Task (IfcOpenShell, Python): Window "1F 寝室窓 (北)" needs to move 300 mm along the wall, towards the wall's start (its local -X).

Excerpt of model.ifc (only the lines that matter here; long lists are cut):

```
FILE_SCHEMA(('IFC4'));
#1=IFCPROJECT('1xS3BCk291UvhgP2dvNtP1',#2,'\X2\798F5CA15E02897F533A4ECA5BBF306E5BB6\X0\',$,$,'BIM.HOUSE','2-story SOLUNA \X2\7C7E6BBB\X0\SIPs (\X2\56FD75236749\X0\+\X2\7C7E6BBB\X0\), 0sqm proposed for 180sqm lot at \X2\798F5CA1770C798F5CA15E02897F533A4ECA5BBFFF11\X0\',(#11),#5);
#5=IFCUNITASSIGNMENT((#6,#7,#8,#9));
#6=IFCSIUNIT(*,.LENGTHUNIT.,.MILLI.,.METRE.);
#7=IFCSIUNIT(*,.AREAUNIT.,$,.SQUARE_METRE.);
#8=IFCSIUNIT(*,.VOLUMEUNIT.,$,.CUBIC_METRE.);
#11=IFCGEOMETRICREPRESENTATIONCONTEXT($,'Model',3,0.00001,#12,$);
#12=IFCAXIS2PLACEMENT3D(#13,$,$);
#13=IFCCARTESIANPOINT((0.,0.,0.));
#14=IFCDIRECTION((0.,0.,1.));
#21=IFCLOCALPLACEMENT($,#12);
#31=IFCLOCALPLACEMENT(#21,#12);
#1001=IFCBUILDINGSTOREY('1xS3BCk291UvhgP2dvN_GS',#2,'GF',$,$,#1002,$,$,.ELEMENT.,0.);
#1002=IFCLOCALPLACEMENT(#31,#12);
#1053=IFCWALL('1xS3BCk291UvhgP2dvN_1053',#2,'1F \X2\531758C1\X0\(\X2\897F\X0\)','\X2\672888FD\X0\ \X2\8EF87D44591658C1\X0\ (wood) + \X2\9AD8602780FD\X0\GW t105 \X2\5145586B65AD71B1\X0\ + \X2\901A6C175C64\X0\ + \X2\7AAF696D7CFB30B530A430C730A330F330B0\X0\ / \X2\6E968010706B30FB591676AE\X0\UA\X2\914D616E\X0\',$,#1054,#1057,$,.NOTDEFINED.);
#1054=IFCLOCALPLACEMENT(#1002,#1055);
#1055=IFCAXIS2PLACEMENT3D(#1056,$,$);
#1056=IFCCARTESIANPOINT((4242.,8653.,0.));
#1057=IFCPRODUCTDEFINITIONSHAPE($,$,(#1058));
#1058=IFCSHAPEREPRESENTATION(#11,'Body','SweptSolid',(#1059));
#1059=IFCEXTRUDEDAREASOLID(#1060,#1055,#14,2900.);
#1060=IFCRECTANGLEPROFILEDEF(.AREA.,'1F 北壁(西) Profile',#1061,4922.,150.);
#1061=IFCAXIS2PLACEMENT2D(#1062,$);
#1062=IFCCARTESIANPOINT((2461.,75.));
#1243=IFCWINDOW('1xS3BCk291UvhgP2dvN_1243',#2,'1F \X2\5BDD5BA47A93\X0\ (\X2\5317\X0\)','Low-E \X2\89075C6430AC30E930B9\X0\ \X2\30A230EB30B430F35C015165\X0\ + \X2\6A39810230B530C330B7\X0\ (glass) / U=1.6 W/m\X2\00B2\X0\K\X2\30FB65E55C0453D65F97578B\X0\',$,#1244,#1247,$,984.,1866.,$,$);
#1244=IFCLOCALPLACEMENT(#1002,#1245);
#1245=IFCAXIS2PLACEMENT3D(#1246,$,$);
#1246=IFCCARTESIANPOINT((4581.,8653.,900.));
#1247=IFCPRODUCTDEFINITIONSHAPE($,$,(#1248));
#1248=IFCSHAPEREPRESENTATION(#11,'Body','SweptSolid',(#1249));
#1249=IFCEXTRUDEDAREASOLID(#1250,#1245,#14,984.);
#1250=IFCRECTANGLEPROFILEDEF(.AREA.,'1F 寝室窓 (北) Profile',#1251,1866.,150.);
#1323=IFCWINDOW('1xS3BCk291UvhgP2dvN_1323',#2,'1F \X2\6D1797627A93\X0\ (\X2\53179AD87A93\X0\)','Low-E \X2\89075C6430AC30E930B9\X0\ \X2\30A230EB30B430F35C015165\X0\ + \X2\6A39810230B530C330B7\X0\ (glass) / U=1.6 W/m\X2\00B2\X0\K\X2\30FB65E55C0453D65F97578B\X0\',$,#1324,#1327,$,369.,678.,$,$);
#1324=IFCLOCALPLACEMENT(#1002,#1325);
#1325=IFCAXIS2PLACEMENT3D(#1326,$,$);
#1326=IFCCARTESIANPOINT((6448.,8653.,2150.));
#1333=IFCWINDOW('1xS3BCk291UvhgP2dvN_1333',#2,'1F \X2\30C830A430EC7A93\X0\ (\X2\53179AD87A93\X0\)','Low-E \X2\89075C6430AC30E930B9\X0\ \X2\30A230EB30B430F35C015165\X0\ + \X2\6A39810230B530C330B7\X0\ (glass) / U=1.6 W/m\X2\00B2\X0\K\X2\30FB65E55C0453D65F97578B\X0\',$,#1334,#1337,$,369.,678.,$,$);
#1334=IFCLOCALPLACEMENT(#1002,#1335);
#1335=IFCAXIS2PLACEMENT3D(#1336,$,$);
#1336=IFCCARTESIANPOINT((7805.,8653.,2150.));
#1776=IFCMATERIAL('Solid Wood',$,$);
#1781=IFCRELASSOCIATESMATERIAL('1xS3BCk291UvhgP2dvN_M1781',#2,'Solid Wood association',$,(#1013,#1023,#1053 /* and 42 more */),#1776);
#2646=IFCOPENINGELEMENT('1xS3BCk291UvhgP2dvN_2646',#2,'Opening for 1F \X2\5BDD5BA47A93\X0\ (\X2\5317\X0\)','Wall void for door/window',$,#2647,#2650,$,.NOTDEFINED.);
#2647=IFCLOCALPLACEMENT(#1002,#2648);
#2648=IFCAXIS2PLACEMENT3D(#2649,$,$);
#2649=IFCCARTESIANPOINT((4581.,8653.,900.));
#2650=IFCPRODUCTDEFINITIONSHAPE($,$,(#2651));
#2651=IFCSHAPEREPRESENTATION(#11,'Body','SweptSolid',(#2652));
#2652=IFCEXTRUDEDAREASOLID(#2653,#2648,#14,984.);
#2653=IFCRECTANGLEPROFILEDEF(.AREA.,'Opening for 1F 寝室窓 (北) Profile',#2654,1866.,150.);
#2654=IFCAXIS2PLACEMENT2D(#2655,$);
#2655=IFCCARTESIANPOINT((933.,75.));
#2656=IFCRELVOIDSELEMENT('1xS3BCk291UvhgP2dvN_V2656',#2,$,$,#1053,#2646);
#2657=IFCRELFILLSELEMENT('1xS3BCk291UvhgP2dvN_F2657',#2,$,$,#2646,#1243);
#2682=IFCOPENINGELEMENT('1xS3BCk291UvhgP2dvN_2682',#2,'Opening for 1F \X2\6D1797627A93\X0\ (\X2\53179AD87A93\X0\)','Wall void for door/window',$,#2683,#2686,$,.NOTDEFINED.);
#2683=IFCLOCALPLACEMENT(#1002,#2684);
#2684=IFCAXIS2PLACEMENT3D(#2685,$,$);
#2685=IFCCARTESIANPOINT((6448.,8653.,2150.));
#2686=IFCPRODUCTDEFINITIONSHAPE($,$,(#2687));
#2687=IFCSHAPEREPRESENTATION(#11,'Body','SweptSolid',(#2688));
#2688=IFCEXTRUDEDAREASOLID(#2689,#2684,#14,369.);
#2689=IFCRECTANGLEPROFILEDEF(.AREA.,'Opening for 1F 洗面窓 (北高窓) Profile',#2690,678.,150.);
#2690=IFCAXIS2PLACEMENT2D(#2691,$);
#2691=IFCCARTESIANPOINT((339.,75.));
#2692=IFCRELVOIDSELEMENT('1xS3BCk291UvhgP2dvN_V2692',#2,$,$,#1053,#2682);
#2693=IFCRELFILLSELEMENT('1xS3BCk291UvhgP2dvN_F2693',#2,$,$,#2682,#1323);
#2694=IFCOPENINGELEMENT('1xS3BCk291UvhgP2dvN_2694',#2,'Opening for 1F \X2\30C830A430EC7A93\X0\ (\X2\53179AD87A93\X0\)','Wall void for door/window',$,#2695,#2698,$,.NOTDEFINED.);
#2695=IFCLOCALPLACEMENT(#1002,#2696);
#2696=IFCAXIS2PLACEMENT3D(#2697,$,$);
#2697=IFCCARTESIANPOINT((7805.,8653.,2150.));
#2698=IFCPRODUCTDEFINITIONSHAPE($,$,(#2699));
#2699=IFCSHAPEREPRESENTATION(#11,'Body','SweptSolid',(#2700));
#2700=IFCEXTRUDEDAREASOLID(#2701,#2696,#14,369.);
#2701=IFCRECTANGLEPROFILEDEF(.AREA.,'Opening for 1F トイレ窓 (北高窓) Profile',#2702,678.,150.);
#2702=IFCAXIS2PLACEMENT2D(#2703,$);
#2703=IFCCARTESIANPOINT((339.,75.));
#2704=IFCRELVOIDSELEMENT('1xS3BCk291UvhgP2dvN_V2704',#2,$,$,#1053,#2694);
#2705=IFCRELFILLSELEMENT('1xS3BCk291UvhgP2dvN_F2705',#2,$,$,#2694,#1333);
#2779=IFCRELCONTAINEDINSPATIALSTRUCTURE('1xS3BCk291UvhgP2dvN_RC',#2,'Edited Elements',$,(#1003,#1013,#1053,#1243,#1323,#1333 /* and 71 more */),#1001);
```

```python
import ifcopenshell
import ifcopenshell.api.geometry
import ifcopenshell.util.placement
import ifcopenshell.util.unit

model = ifcopenshell.open("model.ifc")
unit_scale = ifcopenshell.util.unit.calculate_unit_scale(model)

window = model.by_id(1243)
opening = window.FillsVoids[0].RelatingOpeningElement
wall = opening.VoidsElements[0].RelatingBuildingElement

wall_matrix = ifcopenshell.util.placement.get_local_placement(wall.ObjectPlacement)
shift = wall_matrix[:3, 0] * -0.3 / unit_scale
before = ifcopenshell.util.placement.get_local_placement(window.ObjectPlacement)[:3, 3].copy()

# The window is not placed relative to its opening, so move both.
for product in (opening, window):
    matrix = ifcopenshell.util.placement.get_local_placement(product.ObjectPlacement)
    matrix[:3, 3] += shift
    ifcopenshell.api.geometry.edit_object_placement(model, product=product, matrix=matrix, is_si=False)

after = ifcopenshell.util.placement.get_local_placement(window.ObjectPlacement)[:3, 3]
print("window moved by", (after - before).round(3) + 0.0)

model.write("model_updated.ifc")
```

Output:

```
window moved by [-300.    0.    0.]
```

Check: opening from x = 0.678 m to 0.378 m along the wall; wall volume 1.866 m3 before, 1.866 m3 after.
